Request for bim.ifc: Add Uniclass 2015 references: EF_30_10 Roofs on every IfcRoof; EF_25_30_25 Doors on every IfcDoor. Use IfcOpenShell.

First a look at what the model holds.

```python
import ifcopenshell

model = ifcopenshell.open("bim.ifc")
print(model.schema)
print("classifications:", [c.Name for c in model.by_type("IfcClassification")])
for ifc_class in ("IfcDoor", "IfcRoof", "IfcStair", "IfcWall", "IfcWindow"):
    print(ifc_class, len(model.by_type(ifc_class)))
```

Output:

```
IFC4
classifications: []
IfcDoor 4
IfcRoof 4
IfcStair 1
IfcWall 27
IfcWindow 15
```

```python
import ifcopenshell
import ifcopenshell.api.classification

model = ifcopenshell.open("bim.ifc")

system = ifcopenshell.api.classification.add_classification(model, classification="Uniclass 2015")

codes = {
    "IfcRoof": ("EF_30_10", "Roofs"),
    "IfcDoor": ("EF_25_30_25", "Doors"),
}
for ifc_class, (code, name) in codes.items():
    products = model.by_type(ifc_class)
    ifcopenshell.api.classification.add_reference(
        model, products=products, classification=system, identification=code, name=name
    )
    print(code, len(products))

model.write("bim_rev.ifc")
```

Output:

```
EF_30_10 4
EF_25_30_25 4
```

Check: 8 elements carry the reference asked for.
